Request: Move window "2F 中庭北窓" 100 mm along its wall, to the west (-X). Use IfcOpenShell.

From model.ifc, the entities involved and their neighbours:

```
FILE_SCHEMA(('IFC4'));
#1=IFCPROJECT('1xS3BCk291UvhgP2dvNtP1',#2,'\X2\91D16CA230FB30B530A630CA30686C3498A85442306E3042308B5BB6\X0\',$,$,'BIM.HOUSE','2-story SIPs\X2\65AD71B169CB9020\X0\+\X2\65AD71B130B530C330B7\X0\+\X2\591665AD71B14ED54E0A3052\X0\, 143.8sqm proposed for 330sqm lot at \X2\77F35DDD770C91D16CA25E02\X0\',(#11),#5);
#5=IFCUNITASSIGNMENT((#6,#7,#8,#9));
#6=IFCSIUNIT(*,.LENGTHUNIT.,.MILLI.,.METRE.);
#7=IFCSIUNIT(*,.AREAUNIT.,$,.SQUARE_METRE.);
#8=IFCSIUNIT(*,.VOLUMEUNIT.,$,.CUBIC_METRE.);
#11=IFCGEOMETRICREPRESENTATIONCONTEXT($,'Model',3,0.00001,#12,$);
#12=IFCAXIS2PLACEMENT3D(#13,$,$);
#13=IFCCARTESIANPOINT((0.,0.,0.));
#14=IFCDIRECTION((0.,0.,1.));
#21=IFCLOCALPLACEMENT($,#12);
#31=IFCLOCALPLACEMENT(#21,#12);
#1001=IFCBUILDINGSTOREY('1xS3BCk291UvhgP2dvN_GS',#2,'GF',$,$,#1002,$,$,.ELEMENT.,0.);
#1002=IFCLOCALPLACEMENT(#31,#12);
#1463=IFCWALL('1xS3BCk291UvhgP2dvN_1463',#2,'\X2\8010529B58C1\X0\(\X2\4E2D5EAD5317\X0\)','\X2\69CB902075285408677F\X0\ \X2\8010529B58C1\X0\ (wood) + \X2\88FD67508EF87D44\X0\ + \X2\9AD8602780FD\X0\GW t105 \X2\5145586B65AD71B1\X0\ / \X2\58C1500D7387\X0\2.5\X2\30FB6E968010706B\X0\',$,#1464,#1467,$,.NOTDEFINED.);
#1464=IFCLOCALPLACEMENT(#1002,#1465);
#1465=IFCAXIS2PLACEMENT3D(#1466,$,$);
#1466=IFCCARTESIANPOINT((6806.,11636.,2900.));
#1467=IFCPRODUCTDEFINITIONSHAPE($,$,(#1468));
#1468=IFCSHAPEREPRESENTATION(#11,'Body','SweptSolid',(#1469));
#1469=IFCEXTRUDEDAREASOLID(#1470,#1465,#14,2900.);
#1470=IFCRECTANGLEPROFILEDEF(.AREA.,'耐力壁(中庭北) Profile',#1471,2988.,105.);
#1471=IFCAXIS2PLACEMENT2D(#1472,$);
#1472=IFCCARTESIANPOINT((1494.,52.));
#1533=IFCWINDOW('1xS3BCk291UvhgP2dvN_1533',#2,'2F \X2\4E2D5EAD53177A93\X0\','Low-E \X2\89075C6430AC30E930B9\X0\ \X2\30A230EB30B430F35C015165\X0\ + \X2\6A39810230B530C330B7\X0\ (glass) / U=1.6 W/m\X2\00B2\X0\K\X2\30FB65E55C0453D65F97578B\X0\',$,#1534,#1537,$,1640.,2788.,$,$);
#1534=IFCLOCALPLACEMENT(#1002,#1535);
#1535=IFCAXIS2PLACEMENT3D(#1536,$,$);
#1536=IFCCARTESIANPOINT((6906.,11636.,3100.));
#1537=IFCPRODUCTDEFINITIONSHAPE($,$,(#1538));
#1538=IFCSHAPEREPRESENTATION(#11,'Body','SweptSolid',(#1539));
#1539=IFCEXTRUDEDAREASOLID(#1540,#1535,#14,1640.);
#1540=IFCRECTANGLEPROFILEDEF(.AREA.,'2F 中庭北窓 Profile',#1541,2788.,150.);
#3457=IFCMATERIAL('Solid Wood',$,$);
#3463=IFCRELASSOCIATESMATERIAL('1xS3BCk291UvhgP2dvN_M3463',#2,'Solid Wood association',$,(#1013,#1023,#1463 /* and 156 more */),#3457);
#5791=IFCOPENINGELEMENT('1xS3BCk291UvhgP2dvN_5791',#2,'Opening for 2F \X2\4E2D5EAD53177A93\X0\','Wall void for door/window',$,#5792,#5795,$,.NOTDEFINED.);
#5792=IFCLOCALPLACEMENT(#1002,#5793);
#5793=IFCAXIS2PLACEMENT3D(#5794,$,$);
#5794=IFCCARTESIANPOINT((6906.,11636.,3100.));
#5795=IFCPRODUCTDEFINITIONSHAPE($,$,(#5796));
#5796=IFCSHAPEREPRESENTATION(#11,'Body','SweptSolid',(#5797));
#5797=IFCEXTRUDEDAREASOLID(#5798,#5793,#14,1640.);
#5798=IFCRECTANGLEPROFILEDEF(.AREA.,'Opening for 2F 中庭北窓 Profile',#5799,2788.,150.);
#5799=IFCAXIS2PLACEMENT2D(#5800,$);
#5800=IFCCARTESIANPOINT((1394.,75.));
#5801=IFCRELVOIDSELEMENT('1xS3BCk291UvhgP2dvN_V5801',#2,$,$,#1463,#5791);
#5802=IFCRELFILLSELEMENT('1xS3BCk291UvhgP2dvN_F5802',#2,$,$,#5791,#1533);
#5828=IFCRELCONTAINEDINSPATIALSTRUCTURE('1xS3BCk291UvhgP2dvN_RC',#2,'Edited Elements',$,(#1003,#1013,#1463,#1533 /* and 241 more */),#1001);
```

```python
import ifcopenshell
import ifcopenshell.api.geometry
import ifcopenshell.util.placement
import ifcopenshell.util.unit

model = ifcopenshell.open("model.ifc")
unit_scale = ifcopenshell.util.unit.calculate_unit_scale(model)

window = model.by_guid("1xS3BCk291UvhgP2dvN_1533")
opening = window.FillsVoids[0].RelatingOpeningElement
wall = opening.VoidsElements[0].RelatingBuildingElement

wall_matrix = ifcopenshell.util.placement.get_local_placement(wall.ObjectPlacement)
shift = wall_matrix[:3, 0] * -0.1 / unit_scale
before = ifcopenshell.util.placement.get_local_placement(window.ObjectPlacement)[:3, 3].copy()

# The window is not placed relative to its opening, so move both.
for product in (opening, window):
    matrix = ifcopenshell.util.placement.get_local_placement(product.ObjectPlacement)
    matrix[:3, 3] += shift
    ifcopenshell.api.geometry.edit_object_placement(model, product=product, matrix=matrix, is_si=False)

after = ifcopenshell.util.placement.get_local_placement(window.ObjectPlacement)[:3, 3]
print("window moved by", (after - before).round(3) + 0.0)

model.write("model_edited.ifc")
```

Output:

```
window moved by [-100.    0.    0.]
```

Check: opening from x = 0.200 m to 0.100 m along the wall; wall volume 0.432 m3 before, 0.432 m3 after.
